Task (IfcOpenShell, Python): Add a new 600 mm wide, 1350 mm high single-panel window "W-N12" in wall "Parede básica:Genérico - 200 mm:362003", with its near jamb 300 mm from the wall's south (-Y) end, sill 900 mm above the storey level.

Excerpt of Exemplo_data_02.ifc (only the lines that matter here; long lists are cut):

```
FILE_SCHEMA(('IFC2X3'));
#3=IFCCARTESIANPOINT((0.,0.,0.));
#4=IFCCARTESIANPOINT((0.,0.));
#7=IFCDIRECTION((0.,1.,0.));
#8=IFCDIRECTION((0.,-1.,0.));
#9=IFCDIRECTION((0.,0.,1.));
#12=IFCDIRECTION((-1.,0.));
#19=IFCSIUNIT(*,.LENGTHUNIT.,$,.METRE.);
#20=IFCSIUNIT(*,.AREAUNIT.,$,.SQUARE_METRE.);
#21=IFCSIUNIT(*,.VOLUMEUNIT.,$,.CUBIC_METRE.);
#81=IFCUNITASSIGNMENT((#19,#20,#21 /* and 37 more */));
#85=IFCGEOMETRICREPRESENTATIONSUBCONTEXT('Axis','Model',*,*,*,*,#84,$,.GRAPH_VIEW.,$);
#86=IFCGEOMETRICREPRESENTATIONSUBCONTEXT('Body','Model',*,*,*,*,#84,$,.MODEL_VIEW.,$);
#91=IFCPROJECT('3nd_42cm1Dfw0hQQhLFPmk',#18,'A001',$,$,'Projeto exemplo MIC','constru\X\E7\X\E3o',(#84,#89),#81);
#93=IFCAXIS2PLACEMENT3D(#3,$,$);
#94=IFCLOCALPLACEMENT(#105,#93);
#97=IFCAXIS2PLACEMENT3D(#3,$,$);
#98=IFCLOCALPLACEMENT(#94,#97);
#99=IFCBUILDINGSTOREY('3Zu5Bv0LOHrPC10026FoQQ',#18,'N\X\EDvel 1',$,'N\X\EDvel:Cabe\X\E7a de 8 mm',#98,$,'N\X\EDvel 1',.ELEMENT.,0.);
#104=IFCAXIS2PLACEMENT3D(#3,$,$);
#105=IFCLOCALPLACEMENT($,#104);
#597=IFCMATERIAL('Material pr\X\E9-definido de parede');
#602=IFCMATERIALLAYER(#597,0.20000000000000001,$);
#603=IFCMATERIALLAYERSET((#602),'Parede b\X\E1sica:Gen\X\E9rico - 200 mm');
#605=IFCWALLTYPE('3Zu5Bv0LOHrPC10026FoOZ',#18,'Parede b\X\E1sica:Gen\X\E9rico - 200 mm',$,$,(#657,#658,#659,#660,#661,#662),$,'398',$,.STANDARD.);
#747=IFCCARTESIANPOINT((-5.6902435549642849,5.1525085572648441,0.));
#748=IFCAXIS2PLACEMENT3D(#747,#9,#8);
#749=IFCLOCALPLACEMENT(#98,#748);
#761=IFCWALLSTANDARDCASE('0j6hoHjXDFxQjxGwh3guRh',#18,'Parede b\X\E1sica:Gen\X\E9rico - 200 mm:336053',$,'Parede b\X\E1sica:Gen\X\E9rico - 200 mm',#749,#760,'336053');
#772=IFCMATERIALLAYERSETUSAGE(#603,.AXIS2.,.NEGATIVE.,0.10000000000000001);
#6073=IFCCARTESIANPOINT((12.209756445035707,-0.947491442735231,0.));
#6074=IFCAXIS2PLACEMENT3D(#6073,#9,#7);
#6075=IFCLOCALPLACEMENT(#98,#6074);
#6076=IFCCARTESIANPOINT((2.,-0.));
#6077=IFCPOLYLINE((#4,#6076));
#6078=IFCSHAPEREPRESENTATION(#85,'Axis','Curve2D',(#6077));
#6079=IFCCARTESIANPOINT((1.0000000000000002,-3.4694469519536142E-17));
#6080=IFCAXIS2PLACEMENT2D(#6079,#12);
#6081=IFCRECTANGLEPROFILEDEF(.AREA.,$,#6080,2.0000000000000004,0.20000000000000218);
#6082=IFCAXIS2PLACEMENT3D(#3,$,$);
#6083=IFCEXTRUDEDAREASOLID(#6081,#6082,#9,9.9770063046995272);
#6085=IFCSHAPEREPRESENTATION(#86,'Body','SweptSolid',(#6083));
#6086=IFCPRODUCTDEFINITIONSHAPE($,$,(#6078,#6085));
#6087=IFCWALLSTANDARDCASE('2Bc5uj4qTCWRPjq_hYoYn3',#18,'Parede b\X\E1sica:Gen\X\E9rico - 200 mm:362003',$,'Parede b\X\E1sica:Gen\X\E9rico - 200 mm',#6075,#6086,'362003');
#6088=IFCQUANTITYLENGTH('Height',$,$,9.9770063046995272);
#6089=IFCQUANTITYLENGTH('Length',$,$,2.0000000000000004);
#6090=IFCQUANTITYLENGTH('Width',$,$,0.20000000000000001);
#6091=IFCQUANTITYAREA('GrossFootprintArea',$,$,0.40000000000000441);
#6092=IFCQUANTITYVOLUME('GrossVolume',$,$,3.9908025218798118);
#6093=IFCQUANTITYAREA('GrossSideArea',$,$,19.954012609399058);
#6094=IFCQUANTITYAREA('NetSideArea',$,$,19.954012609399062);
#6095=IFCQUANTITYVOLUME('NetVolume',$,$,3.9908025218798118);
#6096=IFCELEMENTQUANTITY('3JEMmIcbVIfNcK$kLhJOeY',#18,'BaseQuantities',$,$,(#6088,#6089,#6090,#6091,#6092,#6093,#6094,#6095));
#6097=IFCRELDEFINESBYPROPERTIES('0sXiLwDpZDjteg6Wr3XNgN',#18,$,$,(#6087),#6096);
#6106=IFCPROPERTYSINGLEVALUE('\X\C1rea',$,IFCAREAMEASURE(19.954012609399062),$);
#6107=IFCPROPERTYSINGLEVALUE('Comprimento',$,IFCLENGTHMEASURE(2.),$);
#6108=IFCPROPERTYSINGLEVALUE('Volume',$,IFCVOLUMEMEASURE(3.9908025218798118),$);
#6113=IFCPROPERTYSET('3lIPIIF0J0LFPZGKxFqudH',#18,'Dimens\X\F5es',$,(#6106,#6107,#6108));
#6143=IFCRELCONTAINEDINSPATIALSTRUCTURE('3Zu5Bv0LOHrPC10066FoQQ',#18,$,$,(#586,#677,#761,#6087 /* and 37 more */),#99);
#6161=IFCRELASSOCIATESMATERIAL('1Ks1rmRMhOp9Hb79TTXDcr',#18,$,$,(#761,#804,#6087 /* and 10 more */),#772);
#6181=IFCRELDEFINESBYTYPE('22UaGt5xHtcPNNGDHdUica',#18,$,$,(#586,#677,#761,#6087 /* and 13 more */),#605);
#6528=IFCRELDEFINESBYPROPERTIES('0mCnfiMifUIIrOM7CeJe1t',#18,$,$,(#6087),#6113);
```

```python
import numpy as np
import ifcopenshell
import ifcopenshell.api.feature
import ifcopenshell.api.geometry
import ifcopenshell.api.pset
import ifcopenshell.api.root
import ifcopenshell.api.spatial
import ifcopenshell.api.type
import ifcopenshell.geom
import ifcopenshell.util.element
import ifcopenshell.util.placement
import ifcopenshell.util.representation
import ifcopenshell.util.shape
import ifcopenshell.util.unit

model = ifcopenshell.open("Exemplo_data_02.ifc")
unit_scale = ifcopenshell.util.unit.calculate_unit_scale(model)
area_scale = ifcopenshell.util.unit.calculate_unit_scale(model, "AREAUNIT")
volume_scale = ifcopenshell.util.unit.calculate_unit_scale(model, "VOLUMEUNIT")
settings = ifcopenshell.geom.settings()


def volume(element):
    """Net volume in cubic metres, openings subtracted."""
    shape = ifcopenshell.geom.create_shape(settings, element)
    return ifcopenshell.util.shape.get_volume(shape.geometry)


wall = model.by_guid("2Bc5uj4qTCWRPjq_hYoYn3")
storey = ifcopenshell.util.element.get_container(wall, ifc_class="IfcBuildingStorey")
context = ifcopenshell.util.representation.get_context(model, "Model", "Body", "MODEL_VIEW")
before = volume(wall)

width, height, from_end, sill = 0.6, 1.35, 0.3, 0.9  # metres

# The wall runs along its own X axis, and the end named is its -X end.
wall_shape = ifcopenshell.geom.create_shape(settings, wall)
x, y, z = ifcopenshell.util.shape.get_vertices(wall_shape.geometry).T
start = x.min() + from_end
face, thickness = float(y.min()), float(y.max() - y.min())
wall_matrix = ifcopenshell.util.placement.get_local_placement(wall.ObjectPlacement)
level = ifcopenshell.util.placement.get_local_placement(storey.ObjectPlacement)[2, 3]


def in_wall(x, y):
    """Placement at x, y metres in the wall's axes, at sill height."""
    matrix = wall_matrix.copy()
    matrix[:, 3] = wall_matrix @ np.array([x / unit_scale, y / unit_scale, 0.0, 1.0])
    matrix[2, 3] = level + sill / unit_scale
    return matrix


# Opening: a box that overshoots both wall faces by 50 mm.
opening = ifcopenshell.api.root.create_entity(model, ifc_class="IfcOpeningElement")
box = ifcopenshell.api.geometry.add_wall_representation(
    model, context=context, length=width, height=height, thickness=thickness + 0.1
)
ifcopenshell.api.geometry.assign_representation(model, product=opening, representation=box)
ifcopenshell.api.geometry.edit_object_placement(model, product=opening, matrix=in_wall(start, face - 0.05), is_si=False)
ifcopenshell.api.feature.add_feature(model, feature=opening, element=wall)

window = ifcopenshell.api.root.create_entity(model, ifc_class="IfcWindow", name="W-N12")
window.OverallWidth, window.OverallHeight = width / unit_scale, height / unit_scale
body = ifcopenshell.api.geometry.add_window_representation(
    model,
    context=context,
    overall_width=window.OverallWidth,
    overall_height=window.OverallHeight,
    partition_type="SINGLE_PANEL",
)
ifcopenshell.api.geometry.assign_representation(model, product=window, representation=body)
ifcopenshell.api.spatial.assign_container(model, products=[window], relating_structure=storey)
fills = ifcopenshell.api.feature.add_filling(model, opening=opening, element=window)
fills.OwnerHistory = window.OwnerHistory  # required in IFC2X3

# IFC2X3 keeps the operation on the window style.
style = ifcopenshell.api.root.create_entity(model, ifc_class="IfcWindowStyle", name="W-N12")
style.OperationType, style.ConstructionType = "SINGLE_PANEL", "NOTDEFINED"
style.ParameterTakesPrecedence = style.Sizeable = False
ifcopenshell.api.type.assign_type(model, related_objects=[window], relating_type=style)

# Centre the window in the wall's thickness.
ifcopenshell.api.geometry.edit_object_placement(model, product=window, matrix=in_wall(start, face), is_si=False)
window_shape = ifcopenshell.geom.create_shape(settings, window)
depth = ifcopenshell.util.shape.get_vertices(window_shape.geometry)[:, 1]
offset = face + thickness / 2 - (depth.min() + depth.max()) / 2
ifcopenshell.api.geometry.edit_object_placement(model, product=window, matrix=in_wall(start, offset), is_si=False)

after = volume(wall)

# Update the wall's stored quantities.
qto = model.by_id(ifcopenshell.util.element.get_pset(wall, "BaseQuantities", should_inherit=False)["id"])
ifcopenshell.api.pset.edit_qto(model, qto=qto, properties={
    "NetSideArea": after / thickness / area_scale,
    "NetVolume": after / volume_scale,
})
pset = model.by_id(ifcopenshell.util.element.get_pset(wall, "Dimensões", should_inherit=False)["id"])
ifcopenshell.api.pset.edit_pset(model, pset=pset, properties={
    "Área": model.create_entity("IfcAreaMeasure", after / thickness / area_scale),
    "Volume": model.create_entity("IfcVolumeMeasure", after / volume_scale),
})

print(f"wall volume {before:.3f} -> {after:.3f} m3")

model.write("Exemplo_data_02_v2.ifc")
```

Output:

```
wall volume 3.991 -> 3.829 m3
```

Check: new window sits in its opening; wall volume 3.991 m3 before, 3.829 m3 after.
